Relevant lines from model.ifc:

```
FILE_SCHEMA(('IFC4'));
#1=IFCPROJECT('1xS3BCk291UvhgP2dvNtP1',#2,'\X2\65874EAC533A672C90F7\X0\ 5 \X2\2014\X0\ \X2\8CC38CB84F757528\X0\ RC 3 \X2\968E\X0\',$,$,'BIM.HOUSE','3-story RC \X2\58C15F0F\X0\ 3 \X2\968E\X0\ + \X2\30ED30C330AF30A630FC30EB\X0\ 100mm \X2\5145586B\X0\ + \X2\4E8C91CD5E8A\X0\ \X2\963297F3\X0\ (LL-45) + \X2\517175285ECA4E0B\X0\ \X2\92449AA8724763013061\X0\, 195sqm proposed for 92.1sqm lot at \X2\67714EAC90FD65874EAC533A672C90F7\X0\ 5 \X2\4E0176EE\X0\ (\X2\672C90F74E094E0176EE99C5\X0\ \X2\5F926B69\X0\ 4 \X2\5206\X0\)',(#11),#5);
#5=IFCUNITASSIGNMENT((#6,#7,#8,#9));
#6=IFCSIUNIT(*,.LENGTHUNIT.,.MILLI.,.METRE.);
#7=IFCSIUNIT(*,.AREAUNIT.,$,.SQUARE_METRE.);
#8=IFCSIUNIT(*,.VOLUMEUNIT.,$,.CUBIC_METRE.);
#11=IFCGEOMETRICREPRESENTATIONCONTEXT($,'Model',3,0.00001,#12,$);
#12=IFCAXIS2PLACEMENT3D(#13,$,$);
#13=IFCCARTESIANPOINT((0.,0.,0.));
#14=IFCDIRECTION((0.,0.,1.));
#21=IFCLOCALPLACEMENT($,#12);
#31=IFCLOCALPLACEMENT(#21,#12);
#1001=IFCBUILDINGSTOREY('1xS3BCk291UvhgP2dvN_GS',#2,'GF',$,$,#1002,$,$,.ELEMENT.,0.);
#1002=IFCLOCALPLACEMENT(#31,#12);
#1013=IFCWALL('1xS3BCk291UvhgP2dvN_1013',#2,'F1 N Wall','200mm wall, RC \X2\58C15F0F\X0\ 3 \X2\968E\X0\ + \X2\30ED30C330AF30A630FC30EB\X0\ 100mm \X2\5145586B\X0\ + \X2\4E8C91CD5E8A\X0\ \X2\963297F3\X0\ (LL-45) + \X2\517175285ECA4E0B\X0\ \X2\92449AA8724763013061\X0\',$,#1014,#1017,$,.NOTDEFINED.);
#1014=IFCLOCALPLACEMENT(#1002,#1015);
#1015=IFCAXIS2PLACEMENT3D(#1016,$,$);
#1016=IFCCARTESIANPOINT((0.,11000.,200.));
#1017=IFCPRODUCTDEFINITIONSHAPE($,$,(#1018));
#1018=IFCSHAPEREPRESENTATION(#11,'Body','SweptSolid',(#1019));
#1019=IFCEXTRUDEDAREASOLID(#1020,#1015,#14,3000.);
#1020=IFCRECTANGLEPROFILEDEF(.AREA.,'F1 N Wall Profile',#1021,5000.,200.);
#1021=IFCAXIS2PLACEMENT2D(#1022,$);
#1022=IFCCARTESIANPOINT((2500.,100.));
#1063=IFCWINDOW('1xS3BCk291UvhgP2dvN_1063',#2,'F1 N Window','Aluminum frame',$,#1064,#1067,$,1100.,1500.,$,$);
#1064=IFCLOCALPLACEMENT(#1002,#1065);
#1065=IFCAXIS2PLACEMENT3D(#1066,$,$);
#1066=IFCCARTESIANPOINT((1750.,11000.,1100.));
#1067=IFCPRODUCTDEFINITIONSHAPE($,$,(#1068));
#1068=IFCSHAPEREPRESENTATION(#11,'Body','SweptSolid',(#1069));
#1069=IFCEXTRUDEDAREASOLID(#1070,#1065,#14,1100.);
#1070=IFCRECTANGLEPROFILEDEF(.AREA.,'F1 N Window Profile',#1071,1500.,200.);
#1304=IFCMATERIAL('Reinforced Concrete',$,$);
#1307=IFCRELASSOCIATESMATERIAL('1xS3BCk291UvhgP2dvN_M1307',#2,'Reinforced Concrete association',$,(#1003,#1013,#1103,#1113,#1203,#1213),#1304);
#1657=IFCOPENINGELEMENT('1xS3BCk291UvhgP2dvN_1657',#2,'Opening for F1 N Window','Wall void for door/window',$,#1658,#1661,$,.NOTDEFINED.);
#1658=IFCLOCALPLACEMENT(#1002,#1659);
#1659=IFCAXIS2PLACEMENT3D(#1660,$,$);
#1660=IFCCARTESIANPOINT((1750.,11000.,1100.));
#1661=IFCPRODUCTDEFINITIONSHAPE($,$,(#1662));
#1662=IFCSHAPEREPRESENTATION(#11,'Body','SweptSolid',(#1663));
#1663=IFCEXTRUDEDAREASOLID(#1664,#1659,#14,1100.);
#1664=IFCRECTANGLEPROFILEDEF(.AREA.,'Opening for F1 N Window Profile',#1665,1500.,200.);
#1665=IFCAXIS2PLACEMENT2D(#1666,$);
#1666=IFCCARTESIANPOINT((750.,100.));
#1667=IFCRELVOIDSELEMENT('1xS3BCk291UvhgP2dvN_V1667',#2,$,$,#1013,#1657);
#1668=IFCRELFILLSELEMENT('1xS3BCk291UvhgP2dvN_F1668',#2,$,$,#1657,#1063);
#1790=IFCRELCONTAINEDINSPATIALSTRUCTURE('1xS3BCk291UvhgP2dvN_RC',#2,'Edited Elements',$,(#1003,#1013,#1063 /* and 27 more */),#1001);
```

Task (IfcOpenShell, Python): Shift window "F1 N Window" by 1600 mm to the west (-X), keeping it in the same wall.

```python
import ifcopenshell
import ifcopenshell.api.geometry
import ifcopenshell.util.placement

model = ifcopenshell.open("model.ifc")

window = model.by_id(1063)
opening = window.FillsVoids[0].RelatingOpeningElement
wall = opening.VoidsElements[0].RelatingBuildingElement

wall_matrix = ifcopenshell.util.placement.get_local_placement(wall.ObjectPlacement)
shift = wall_matrix[:3, 0] * -1600.0
before = ifcopenshell.util.placement.get_local_placement(window.ObjectPlacement)[:3, 3].copy()

# The window is not placed relative to its opening, so move both.
for product in (opening, window):
    matrix = ifcopenshell.util.placement.get_local_placement(product.ObjectPlacement)
    matrix[:3, 3] += shift
    ifcopenshell.api.geometry.edit_object_placement(model, product=product, matrix=matrix, is_si=False)

after = ifcopenshell.util.placement.get_local_placement(window.ObjectPlacement)[:3, 3]
print("window moved by", (after - before).round(3) + 0.0)

model.write("model_v2.ifc")
```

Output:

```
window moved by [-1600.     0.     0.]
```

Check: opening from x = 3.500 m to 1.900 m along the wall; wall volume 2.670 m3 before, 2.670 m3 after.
